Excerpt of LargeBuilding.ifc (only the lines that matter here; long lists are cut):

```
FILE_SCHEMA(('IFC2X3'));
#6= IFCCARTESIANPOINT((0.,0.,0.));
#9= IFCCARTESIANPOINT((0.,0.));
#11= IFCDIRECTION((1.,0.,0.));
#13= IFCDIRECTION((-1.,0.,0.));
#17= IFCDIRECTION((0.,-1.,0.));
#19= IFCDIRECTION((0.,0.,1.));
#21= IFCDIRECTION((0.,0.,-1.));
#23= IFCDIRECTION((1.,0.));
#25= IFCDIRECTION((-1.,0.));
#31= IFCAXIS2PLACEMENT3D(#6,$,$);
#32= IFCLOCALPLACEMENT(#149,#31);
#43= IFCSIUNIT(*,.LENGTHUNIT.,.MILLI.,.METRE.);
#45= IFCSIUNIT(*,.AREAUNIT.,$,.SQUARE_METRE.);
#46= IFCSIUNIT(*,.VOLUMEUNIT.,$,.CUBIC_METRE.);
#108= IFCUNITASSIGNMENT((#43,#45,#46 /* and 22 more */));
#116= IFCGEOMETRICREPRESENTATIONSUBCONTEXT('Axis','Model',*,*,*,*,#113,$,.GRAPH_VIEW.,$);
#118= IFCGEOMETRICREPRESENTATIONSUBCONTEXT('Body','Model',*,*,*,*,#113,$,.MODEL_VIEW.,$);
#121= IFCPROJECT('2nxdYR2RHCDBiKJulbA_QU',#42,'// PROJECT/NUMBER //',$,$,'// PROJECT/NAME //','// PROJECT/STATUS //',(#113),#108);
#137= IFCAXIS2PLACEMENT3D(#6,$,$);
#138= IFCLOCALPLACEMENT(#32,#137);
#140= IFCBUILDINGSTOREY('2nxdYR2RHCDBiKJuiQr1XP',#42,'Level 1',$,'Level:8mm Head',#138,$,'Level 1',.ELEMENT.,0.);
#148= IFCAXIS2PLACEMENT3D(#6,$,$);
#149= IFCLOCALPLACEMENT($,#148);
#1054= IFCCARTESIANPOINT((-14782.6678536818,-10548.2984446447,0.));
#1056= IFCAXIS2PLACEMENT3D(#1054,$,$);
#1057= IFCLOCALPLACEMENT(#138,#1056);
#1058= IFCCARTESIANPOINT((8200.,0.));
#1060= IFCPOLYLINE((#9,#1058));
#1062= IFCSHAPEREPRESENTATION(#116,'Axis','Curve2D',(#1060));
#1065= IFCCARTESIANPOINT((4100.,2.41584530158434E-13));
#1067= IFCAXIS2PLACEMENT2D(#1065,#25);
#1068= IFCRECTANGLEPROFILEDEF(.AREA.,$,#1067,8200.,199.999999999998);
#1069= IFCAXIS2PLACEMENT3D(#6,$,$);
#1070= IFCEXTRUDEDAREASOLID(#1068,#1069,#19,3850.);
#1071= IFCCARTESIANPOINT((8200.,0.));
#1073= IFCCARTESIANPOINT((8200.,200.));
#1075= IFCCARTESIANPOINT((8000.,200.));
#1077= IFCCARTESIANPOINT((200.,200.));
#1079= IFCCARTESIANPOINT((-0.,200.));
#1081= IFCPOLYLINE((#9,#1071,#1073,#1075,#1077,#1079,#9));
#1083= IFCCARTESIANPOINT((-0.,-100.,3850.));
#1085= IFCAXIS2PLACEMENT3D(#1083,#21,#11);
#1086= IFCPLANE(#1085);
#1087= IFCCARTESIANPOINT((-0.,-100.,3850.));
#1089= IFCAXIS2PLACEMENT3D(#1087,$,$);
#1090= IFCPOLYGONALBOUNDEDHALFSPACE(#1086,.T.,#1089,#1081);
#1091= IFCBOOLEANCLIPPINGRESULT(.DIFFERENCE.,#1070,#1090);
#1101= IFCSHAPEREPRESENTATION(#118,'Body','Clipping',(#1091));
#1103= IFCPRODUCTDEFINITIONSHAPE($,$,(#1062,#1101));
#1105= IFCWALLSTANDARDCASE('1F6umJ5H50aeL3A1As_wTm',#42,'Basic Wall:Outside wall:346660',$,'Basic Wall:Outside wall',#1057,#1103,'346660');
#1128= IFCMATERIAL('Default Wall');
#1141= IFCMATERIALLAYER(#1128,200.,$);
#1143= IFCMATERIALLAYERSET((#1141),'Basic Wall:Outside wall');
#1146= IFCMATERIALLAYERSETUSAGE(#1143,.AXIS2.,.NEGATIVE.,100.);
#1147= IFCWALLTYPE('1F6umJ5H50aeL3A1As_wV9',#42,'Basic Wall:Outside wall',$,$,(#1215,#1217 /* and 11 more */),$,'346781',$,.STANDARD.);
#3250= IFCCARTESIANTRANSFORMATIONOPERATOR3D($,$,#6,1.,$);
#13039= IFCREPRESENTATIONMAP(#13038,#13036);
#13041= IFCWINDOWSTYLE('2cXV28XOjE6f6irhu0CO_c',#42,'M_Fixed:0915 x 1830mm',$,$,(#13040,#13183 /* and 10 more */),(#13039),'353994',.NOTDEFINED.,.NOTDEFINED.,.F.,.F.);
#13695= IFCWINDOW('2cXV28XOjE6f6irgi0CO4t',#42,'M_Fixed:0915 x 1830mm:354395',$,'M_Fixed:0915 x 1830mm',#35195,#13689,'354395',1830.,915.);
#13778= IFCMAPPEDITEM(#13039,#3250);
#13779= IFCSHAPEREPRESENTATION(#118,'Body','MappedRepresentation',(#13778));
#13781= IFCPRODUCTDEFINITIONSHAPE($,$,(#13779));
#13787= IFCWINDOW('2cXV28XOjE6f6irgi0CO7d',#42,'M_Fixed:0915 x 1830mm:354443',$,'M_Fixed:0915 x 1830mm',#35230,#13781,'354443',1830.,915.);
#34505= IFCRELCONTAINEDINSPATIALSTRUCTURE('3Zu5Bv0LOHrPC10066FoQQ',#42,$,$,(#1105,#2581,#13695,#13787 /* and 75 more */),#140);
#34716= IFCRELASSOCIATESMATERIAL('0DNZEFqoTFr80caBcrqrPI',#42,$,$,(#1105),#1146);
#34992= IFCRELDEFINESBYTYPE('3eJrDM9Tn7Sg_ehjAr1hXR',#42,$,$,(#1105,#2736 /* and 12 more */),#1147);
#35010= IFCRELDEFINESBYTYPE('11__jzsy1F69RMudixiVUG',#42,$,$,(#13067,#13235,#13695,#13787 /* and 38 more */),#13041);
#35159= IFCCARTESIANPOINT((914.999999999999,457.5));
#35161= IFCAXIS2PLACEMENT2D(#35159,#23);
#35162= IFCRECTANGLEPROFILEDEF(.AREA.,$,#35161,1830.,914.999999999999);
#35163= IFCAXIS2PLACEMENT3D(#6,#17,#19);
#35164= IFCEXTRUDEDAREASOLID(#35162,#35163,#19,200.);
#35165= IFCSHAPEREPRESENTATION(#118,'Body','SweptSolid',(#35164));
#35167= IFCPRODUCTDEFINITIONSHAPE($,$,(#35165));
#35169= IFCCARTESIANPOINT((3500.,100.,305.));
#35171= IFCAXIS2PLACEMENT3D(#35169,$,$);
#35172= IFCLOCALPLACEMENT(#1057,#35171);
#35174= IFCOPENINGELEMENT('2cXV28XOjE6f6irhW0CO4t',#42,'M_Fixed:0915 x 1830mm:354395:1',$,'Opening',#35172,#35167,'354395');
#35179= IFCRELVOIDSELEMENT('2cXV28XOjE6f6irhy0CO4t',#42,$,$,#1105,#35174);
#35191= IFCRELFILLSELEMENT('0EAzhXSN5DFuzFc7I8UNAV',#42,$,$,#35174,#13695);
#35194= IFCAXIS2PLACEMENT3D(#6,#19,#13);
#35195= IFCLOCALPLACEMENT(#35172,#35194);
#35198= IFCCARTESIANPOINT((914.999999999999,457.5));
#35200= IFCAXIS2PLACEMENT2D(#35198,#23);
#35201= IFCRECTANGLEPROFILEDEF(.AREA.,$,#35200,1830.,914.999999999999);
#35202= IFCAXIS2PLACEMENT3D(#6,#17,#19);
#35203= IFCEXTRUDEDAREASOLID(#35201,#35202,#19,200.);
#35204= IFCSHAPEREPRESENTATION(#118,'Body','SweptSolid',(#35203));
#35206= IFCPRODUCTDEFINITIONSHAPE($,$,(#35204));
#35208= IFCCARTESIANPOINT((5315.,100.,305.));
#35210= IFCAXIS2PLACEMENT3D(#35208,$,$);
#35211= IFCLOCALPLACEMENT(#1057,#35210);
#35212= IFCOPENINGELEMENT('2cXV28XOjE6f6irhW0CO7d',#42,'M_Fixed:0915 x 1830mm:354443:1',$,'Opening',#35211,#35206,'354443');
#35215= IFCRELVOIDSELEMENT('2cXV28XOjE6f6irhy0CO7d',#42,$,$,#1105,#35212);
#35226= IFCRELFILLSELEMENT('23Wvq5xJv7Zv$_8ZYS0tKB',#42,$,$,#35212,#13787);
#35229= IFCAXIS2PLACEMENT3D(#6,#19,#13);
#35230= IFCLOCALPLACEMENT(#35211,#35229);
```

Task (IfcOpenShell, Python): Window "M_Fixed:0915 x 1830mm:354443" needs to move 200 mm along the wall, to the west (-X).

```python
import ifcopenshell
import ifcopenshell.api.geometry
import ifcopenshell.util.placement

model = ifcopenshell.open("LargeBuilding.ifc")

window = model.by_guid("2cXV28XOjE6f6irgi0CO7d")
opening = window.FillsVoids[0].RelatingOpeningElement
wall = opening.VoidsElements[0].RelatingBuildingElement

wall_matrix = ifcopenshell.util.placement.get_local_placement(wall.ObjectPlacement)
shift = wall_matrix[:3, 0] * -200.0
before = ifcopenshell.util.placement.get_local_placement(window.ObjectPlacement)[:3, 3].copy()

# The window is placed relative to its opening, so it follows when the opening moves.
matrix = ifcopenshell.util.placement.get_local_placement(opening.ObjectPlacement)
matrix[:3, 3] += shift
ifcopenshell.api.geometry.edit_object_placement(
    model, product=opening, matrix=matrix, is_si=False, should_transform_children=True
)

after = ifcopenshell.util.placement.get_local_placement(window.ObjectPlacement)[:3, 3]
print("window moved by", (after - before).round(3) + 0.0)

model.write("LargeBuilding_updated.ifc")
```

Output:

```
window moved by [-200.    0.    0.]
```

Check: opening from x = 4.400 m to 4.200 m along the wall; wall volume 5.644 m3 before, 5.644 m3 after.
